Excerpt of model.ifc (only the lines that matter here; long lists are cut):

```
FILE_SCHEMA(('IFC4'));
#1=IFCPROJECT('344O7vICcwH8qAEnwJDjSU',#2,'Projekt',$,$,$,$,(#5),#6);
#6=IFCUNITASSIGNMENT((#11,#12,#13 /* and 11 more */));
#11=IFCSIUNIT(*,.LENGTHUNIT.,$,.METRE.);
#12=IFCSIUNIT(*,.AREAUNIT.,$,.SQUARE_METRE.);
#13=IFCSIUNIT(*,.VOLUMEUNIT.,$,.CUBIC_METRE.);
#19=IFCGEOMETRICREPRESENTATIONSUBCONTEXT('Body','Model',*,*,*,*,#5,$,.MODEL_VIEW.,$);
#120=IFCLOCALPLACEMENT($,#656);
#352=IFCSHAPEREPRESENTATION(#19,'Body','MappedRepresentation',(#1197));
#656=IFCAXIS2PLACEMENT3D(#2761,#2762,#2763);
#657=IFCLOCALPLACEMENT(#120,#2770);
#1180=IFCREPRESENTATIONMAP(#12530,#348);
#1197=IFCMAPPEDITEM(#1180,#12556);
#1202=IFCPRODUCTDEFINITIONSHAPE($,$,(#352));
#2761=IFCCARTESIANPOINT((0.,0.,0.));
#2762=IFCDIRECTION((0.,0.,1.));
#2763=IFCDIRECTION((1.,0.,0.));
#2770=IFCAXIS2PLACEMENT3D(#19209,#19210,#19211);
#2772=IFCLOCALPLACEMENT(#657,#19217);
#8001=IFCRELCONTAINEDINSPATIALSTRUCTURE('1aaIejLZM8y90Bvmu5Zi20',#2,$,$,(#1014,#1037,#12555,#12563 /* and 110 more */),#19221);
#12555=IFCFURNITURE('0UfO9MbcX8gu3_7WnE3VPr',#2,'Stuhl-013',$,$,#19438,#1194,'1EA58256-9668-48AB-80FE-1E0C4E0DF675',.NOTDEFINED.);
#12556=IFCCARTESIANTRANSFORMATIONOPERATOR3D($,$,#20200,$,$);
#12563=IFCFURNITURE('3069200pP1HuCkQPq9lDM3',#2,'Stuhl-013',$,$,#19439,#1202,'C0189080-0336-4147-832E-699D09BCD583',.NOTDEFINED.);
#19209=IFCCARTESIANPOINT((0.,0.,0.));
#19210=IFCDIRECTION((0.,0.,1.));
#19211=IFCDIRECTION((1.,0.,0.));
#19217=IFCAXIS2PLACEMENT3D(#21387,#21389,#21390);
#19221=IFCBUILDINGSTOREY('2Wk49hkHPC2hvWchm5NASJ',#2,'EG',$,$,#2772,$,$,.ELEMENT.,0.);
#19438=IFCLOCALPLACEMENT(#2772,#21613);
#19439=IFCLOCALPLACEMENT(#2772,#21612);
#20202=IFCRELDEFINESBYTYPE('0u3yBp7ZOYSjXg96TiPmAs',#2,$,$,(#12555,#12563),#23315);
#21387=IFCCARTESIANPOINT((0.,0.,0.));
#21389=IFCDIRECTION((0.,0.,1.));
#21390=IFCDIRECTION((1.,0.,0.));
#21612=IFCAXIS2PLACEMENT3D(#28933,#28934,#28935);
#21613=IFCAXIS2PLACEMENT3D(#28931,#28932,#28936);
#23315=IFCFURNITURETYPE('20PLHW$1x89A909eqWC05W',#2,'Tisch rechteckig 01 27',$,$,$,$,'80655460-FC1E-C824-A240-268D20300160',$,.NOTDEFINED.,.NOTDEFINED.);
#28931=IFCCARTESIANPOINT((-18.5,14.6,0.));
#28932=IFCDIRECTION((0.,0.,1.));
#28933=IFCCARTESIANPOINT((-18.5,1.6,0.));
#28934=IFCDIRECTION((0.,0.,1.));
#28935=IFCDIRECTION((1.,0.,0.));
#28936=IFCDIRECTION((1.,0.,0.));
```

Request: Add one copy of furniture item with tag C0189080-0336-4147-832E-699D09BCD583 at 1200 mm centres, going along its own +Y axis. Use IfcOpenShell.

```python
import ifcopenshell
import ifcopenshell.api.geometry
import ifcopenshell.api.root
import ifcopenshell.util.element
import ifcopenshell.util.placement
import ifcopenshell.util.unit

model = ifcopenshell.open("model.ifc")
unit_scale = ifcopenshell.util.unit.calculate_unit_scale(model)


def reuse_history(source, copy):
    """copy_class also copies each property set's owner history, people and application; keep the originals."""
    for rel in copy.IsDefinedBy:
        if rel.is_a("IfcRelDefinesByProperties") and (history := rel.RelatingPropertyDefinition.OwnerHistory):
            rel.RelatingPropertyDefinition.OwnerHistory = source.OwnerHistory
            ifcopenshell.util.element.remove_deep2(model, history)


source = model.by_id(12563)
base = ifcopenshell.util.placement.get_local_placement(source.ObjectPlacement)
step = base[:3, 1] * 1.2 / unit_scale

for i in range(1, 2):
    copy = ifcopenshell.api.root.copy_class(model, product=source)
    copy.Representation = ifcopenshell.util.element.copy_deep(
        model, source.Representation, exclude=["IfcGeometricRepresentationContext", "IfcRepresentationMap"]
    )
    copy.Tag = None
    reuse_history(source, copy)
    matrix = base.copy()
    matrix[:3, 3] += i * step
    print("added at", matrix[:3, 3].round(3) + 0.0)
    ifcopenshell.api.geometry.edit_object_placement(model, product=copy, matrix=matrix, is_si=False)

model.write("model_v2.ifc")
```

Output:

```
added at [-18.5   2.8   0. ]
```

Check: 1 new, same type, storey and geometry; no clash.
